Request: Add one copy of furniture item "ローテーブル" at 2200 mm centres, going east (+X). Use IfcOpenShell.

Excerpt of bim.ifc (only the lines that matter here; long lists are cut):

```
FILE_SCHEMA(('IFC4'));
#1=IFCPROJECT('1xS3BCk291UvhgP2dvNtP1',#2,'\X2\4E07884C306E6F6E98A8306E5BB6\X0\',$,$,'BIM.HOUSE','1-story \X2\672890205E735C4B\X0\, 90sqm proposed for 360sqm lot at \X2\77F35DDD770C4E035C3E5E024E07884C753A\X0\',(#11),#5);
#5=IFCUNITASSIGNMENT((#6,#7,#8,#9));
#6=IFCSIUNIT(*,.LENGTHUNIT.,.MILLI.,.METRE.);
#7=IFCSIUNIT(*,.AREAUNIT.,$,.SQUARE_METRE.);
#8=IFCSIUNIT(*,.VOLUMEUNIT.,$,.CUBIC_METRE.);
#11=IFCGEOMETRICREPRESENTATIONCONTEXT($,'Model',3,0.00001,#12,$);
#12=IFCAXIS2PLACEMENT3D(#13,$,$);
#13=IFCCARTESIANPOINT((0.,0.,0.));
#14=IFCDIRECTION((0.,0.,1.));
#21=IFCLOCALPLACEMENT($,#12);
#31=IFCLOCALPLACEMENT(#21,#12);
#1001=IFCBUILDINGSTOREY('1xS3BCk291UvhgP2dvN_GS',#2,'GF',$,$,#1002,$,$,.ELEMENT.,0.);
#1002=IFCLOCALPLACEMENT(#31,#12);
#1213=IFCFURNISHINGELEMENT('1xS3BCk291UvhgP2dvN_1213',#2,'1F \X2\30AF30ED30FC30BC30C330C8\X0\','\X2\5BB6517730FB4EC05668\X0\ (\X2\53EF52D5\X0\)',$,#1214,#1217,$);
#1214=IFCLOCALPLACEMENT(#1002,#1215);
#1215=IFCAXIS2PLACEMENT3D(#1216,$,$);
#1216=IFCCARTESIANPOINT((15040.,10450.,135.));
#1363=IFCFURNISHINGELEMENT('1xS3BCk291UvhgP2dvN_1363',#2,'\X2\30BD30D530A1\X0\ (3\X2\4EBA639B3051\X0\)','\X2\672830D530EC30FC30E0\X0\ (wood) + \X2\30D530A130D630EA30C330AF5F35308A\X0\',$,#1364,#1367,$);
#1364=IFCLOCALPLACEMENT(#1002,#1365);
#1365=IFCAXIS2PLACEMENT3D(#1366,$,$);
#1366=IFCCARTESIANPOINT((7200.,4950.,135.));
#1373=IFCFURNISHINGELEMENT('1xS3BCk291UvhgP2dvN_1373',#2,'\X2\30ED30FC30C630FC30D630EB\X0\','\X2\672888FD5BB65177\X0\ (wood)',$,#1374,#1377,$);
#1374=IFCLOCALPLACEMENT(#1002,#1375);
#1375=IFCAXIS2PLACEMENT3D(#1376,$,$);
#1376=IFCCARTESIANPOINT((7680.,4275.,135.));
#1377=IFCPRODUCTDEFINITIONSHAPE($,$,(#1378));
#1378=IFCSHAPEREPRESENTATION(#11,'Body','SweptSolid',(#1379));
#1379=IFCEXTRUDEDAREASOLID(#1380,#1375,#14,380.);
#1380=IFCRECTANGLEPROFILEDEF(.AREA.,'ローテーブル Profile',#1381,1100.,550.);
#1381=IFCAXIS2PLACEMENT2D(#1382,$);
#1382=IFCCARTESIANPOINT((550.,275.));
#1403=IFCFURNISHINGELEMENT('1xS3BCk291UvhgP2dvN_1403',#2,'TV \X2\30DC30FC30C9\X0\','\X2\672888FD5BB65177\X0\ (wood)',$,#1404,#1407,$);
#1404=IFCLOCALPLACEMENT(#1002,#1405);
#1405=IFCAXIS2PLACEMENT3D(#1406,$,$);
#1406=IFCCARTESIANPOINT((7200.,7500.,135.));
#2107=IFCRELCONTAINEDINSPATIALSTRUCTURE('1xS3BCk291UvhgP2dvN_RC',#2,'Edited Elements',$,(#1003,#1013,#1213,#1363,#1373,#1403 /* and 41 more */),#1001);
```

```python
import numpy as np
import ifcopenshell
import ifcopenshell.api.geometry
import ifcopenshell.api.root
import ifcopenshell.util.element
import ifcopenshell.util.placement
import ifcopenshell.util.unit

model = ifcopenshell.open("bim.ifc")
unit_scale = ifcopenshell.util.unit.calculate_unit_scale(model)


def reuse_history(source, copy):
    """copy_class also copies each property set's owner history, people and application; keep the originals."""
    for rel in copy.IsDefinedBy:
        if rel.is_a("IfcRelDefinesByProperties") and (history := rel.RelatingPropertyDefinition.OwnerHistory):
            rel.RelatingPropertyDefinition.OwnerHistory = source.OwnerHistory
            ifcopenshell.util.element.remove_deep2(model, history)


source = model.by_guid("1xS3BCk291UvhgP2dvN_1373")
base = ifcopenshell.util.placement.get_local_placement(source.ObjectPlacement)
step = np.array([1.0, 0.0, 0.0]) * 2.2 / unit_scale

for i in range(1, 2):
    copy = ifcopenshell.api.root.copy_class(model, product=source)
    copy.Representation = ifcopenshell.util.element.copy_deep(
        model, source.Representation, exclude=["IfcGeometricRepresentationContext", "IfcRepresentationMap"]
    )
    reuse_history(source, copy)
    matrix = base.copy()
    matrix[:3, 3] += i * step
    print("added at", matrix[:3, 3].round(3) + 0.0)
    ifcopenshell.api.geometry.edit_object_placement(model, product=copy, matrix=matrix, is_si=False)

model.write("bim_updated.ifc")
```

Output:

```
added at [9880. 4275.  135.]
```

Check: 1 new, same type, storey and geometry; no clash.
